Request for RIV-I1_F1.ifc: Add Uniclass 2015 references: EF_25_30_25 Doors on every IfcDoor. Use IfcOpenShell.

First a look at what the model holds.

```python
import ifcopenshell

model = ifcopenshell.open("RIV-I1_F1.ifc")
print(model.schema)
print("classifications:", [c.Name for c in model.by_type("IfcClassification")])
for ifc_class in ("IfcDoor", "IfcRoof", "IfcStair", "IfcWall", "IfcWindow"):
    print(ifc_class, len(model.by_type(ifc_class)))
```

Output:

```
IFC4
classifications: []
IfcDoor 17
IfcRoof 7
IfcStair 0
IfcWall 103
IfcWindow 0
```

```python
import ifcopenshell
import ifcopenshell.api.classification

model = ifcopenshell.open("RIV-I1_F1.ifc")

system = ifcopenshell.api.classification.add_classification(model, classification="Uniclass 2015")

codes = {
    "IfcDoor": ("EF_25_30_25", "Doors"),
}
for ifc_class, (code, name) in codes.items():
    products = model.by_type(ifc_class)
    ifcopenshell.api.classification.add_reference(
        model, products=products, classification=system, identification=code, name=name
    )
    print(code, len(products))

model.write("RIV-I1_F1_rev.ifc")
```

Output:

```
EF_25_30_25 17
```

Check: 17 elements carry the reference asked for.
